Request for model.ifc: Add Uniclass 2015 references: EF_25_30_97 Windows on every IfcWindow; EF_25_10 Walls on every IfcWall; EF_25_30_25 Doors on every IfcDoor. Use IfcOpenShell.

First a look at what the model holds.

```python
import ifcopenshell

model = ifcopenshell.open("model.ifc")
print(model.schema)
print("classifications:", [c.Name for c in model.by_type("IfcClassification")])
for ifc_class in ("IfcDoor", "IfcRoof", "IfcStair", "IfcWall", "IfcWindow"):
    print(ifc_class, len(model.by_type(ifc_class)))
```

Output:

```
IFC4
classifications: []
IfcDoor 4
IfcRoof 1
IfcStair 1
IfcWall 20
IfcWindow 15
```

```python
import ifcopenshell
import ifcopenshell.api.classification

model = ifcopenshell.open("model.ifc")

system = ifcopenshell.api.classification.add_classification(model, classification="Uniclass 2015")

codes = {
    "IfcWindow": ("EF_25_30_97", "Windows"),
    "IfcWall": ("EF_25_10", "Walls"),
    "IfcDoor": ("EF_25_30_25", "Doors"),
}
for ifc_class, (code, name) in codes.items():
    products = model.by_type(ifc_class)
    ifcopenshell.api.classification.add_reference(
        model, products=products, classification=system, identification=code, name=name
    )
    print(code, len(products))

model.write("model_rev.ifc")
```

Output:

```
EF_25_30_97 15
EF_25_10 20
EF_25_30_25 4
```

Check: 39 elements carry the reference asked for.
